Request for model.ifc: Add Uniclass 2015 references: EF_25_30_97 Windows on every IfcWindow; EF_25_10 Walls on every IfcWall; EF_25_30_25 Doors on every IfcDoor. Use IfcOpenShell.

First a look at what the model holds.

```python
import ifcopenshell

model = ifcopenshell.open("model.ifc")
print(model.schema)
print("classifications:", [c.Name for c in model.by_type("IfcClassification")])
for ifc_class in ("IfcDoor", "IfcRoof", "IfcStair", "IfcWall", "IfcWindow"):
    print(ifc_class, len(model.by_type(ifc_class)))
```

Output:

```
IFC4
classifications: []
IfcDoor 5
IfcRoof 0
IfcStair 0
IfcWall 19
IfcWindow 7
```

```python
import ifcopenshell
import ifcopenshell.api.classification

model = ifcopenshell.open("model.ifc")

system = ifcopenshell.api.classification.add_classification(model, classification="Uniclass 2015")

codes = {
    "IfcWindow": ("EF_25_30_97", "Windows"),
    "IfcWall": ("EF_25_10", "Walls"),
    "IfcDoor": ("EF_25_30_25", "Doors"),
}
for ifc_class, (code, name) in codes.items():
    products = model.by_type(ifc_class)
    ifcopenshell.api.classification.add_reference(
        model, products=products, classification=system, identification=code, name=name
    )
    print(code, len(products))

model.write("model_updated.ifc")
```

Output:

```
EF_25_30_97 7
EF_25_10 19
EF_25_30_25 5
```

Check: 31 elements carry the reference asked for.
